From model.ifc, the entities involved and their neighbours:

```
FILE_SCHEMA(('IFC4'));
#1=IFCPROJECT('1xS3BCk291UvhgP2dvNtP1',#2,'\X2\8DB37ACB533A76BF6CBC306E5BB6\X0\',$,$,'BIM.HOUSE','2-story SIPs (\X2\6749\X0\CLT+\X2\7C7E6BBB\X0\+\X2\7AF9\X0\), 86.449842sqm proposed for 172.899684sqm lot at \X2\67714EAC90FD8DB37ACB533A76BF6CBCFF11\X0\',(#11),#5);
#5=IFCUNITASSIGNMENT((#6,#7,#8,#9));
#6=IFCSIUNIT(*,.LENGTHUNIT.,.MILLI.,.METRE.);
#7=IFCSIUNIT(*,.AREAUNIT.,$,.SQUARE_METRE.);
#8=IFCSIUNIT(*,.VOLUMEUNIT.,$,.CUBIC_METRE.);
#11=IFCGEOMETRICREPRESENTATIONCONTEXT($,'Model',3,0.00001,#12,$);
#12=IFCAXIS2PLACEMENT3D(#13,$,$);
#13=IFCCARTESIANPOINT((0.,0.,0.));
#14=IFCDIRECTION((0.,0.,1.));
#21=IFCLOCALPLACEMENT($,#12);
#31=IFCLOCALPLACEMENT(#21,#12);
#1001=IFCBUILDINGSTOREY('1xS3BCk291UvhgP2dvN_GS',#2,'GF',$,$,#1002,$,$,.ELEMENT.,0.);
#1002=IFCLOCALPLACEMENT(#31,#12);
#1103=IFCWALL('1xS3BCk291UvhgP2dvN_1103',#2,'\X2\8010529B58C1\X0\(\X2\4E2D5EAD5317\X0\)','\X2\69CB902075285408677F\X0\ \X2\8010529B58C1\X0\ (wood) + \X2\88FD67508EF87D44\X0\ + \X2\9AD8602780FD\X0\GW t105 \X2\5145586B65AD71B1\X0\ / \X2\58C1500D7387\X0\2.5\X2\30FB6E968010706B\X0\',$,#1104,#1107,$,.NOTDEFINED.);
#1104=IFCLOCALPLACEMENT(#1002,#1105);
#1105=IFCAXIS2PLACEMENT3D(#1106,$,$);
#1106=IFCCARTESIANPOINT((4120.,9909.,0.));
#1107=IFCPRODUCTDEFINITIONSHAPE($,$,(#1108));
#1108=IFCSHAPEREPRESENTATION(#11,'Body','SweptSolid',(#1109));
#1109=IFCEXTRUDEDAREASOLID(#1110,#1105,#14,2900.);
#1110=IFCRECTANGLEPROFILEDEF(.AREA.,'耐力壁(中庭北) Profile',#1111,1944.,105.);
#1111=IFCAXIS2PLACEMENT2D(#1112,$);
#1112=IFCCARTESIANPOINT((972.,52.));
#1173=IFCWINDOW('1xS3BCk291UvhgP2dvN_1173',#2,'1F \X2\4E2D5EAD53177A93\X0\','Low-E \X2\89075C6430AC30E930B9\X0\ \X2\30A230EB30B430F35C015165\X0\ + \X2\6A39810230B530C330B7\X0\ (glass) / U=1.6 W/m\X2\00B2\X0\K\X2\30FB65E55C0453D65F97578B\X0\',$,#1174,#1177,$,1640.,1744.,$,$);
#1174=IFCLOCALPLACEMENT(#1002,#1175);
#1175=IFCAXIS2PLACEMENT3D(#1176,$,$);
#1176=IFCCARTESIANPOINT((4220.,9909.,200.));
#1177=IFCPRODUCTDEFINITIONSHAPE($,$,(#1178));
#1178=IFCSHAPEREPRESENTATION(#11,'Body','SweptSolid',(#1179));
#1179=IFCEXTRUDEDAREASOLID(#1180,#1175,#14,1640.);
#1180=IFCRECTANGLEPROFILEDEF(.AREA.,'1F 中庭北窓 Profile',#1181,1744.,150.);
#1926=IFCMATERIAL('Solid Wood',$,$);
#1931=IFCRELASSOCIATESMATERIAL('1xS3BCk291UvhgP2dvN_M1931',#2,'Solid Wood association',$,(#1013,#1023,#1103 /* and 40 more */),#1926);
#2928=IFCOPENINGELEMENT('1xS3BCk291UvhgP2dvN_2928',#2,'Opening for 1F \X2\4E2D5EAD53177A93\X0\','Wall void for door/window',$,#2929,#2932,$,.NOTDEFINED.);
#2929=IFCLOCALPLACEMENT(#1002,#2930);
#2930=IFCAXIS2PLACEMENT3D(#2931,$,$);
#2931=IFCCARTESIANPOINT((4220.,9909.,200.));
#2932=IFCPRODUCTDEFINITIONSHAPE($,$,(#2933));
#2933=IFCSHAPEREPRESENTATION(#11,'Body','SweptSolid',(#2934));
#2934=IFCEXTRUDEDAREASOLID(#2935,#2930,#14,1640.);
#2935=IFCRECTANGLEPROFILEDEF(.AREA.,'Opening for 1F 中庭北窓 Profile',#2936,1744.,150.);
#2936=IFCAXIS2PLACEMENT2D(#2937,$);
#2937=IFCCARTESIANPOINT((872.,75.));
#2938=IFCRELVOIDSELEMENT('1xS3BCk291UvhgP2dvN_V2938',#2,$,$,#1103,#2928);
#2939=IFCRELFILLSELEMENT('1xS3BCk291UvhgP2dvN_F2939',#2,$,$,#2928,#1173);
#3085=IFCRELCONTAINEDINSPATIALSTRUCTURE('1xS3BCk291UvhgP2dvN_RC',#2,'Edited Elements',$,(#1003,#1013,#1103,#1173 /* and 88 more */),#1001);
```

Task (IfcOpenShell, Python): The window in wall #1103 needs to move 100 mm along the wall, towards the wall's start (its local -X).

```python
import ifcopenshell
import ifcopenshell.api.geometry
import ifcopenshell.util.placement
import ifcopenshell.util.unit

model = ifcopenshell.open("model.ifc")
unit_scale = ifcopenshell.util.unit.calculate_unit_scale(model)

window = model.by_guid("1xS3BCk291UvhgP2dvN_1173")
opening = window.FillsVoids[0].RelatingOpeningElement
wall = opening.VoidsElements[0].RelatingBuildingElement

wall_matrix = ifcopenshell.util.placement.get_local_placement(wall.ObjectPlacement)
shift = wall_matrix[:3, 0] * -0.1 / unit_scale
before = ifcopenshell.util.placement.get_local_placement(window.ObjectPlacement)[:3, 3].copy()

# The window is not placed relative to its opening, so move both.
for product in (opening, window):
    matrix = ifcopenshell.util.placement.get_local_placement(product.ObjectPlacement)
    matrix[:3, 3] += shift
    ifcopenshell.api.geometry.edit_object_placement(model, product=product, matrix=matrix, is_si=False)

after = ifcopenshell.util.placement.get_local_placement(window.ObjectPlacement)[:3, 3]
print("window moved by", (after - before).round(3) + 0.0)

model.write("model_v2.ifc")
```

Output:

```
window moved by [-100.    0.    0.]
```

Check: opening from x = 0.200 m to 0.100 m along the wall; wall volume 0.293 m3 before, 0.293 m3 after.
